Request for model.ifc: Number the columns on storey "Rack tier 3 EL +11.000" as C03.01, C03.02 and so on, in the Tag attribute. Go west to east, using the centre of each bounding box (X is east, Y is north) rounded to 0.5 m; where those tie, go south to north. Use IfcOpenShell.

First a look at what the model holds.

```python
import ifcopenshell
import ifcopenshell.util.element
import ifcopenshell.util.placement

model = ifcopenshell.open("model.ifc")
print(model.schema)
storey = next(s for s in model.by_type("IfcBuildingStorey") if s.Name == "Rack tier 3 EL +11.000")
columns = [e for e in ifcopenshell.util.element.get_decomposition(storey) if e.is_a("IfcColumn")]
for e in sorted(columns, key=lambda e: e.id()):
    origin = ifcopenshell.util.placement.get_local_placement(e.ObjectPlacement)[:3, 3]
    print(e.id(), e.Tag, e.Name, origin.round(2) + 0.0, sep=" | ")
```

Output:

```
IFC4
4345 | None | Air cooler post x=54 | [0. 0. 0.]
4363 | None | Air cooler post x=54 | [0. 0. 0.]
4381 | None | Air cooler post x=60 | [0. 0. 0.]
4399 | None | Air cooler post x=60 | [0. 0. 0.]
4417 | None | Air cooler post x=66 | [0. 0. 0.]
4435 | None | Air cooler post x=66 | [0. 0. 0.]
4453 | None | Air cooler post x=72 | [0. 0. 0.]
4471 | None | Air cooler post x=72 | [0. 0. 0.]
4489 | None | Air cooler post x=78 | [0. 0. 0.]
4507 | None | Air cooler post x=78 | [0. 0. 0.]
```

```python
import ifcopenshell
import ifcopenshell.geom
import ifcopenshell.util.element
import ifcopenshell.util.shape

model = ifcopenshell.open("model.ifc")
settings = ifcopenshell.geom.settings()
settings.set("use-world-coords", True)


def centre(element):
    shape = ifcopenshell.geom.create_shape(settings, element)
    return ifcopenshell.util.shape.get_bbox_centroid(shape.geometry)


storey = next(s for s in model.by_type("IfcBuildingStorey") if s.Name == "Rack tier 3 EL +11.000")
columns = [e for e in ifcopenshell.util.element.get_decomposition(storey) if e.is_a("IfcColumn")]

# Insertion points can sit at a corner or the storey origin, so sort by the geometry (in metres).
centres = {e: centre(e) for e in columns}
columns.sort(key=lambda e: (round(centres[e][0] / 0.5), centres[e][1]))

for i, e in enumerate(columns, start=1):
    number = f"C03.{i:02d}"
    e.Tag = number
    print(e.id(), number)

model.write("model-out.ifc")
```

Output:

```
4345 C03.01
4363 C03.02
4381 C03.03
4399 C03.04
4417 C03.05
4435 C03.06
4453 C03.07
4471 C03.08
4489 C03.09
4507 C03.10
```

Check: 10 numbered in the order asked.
